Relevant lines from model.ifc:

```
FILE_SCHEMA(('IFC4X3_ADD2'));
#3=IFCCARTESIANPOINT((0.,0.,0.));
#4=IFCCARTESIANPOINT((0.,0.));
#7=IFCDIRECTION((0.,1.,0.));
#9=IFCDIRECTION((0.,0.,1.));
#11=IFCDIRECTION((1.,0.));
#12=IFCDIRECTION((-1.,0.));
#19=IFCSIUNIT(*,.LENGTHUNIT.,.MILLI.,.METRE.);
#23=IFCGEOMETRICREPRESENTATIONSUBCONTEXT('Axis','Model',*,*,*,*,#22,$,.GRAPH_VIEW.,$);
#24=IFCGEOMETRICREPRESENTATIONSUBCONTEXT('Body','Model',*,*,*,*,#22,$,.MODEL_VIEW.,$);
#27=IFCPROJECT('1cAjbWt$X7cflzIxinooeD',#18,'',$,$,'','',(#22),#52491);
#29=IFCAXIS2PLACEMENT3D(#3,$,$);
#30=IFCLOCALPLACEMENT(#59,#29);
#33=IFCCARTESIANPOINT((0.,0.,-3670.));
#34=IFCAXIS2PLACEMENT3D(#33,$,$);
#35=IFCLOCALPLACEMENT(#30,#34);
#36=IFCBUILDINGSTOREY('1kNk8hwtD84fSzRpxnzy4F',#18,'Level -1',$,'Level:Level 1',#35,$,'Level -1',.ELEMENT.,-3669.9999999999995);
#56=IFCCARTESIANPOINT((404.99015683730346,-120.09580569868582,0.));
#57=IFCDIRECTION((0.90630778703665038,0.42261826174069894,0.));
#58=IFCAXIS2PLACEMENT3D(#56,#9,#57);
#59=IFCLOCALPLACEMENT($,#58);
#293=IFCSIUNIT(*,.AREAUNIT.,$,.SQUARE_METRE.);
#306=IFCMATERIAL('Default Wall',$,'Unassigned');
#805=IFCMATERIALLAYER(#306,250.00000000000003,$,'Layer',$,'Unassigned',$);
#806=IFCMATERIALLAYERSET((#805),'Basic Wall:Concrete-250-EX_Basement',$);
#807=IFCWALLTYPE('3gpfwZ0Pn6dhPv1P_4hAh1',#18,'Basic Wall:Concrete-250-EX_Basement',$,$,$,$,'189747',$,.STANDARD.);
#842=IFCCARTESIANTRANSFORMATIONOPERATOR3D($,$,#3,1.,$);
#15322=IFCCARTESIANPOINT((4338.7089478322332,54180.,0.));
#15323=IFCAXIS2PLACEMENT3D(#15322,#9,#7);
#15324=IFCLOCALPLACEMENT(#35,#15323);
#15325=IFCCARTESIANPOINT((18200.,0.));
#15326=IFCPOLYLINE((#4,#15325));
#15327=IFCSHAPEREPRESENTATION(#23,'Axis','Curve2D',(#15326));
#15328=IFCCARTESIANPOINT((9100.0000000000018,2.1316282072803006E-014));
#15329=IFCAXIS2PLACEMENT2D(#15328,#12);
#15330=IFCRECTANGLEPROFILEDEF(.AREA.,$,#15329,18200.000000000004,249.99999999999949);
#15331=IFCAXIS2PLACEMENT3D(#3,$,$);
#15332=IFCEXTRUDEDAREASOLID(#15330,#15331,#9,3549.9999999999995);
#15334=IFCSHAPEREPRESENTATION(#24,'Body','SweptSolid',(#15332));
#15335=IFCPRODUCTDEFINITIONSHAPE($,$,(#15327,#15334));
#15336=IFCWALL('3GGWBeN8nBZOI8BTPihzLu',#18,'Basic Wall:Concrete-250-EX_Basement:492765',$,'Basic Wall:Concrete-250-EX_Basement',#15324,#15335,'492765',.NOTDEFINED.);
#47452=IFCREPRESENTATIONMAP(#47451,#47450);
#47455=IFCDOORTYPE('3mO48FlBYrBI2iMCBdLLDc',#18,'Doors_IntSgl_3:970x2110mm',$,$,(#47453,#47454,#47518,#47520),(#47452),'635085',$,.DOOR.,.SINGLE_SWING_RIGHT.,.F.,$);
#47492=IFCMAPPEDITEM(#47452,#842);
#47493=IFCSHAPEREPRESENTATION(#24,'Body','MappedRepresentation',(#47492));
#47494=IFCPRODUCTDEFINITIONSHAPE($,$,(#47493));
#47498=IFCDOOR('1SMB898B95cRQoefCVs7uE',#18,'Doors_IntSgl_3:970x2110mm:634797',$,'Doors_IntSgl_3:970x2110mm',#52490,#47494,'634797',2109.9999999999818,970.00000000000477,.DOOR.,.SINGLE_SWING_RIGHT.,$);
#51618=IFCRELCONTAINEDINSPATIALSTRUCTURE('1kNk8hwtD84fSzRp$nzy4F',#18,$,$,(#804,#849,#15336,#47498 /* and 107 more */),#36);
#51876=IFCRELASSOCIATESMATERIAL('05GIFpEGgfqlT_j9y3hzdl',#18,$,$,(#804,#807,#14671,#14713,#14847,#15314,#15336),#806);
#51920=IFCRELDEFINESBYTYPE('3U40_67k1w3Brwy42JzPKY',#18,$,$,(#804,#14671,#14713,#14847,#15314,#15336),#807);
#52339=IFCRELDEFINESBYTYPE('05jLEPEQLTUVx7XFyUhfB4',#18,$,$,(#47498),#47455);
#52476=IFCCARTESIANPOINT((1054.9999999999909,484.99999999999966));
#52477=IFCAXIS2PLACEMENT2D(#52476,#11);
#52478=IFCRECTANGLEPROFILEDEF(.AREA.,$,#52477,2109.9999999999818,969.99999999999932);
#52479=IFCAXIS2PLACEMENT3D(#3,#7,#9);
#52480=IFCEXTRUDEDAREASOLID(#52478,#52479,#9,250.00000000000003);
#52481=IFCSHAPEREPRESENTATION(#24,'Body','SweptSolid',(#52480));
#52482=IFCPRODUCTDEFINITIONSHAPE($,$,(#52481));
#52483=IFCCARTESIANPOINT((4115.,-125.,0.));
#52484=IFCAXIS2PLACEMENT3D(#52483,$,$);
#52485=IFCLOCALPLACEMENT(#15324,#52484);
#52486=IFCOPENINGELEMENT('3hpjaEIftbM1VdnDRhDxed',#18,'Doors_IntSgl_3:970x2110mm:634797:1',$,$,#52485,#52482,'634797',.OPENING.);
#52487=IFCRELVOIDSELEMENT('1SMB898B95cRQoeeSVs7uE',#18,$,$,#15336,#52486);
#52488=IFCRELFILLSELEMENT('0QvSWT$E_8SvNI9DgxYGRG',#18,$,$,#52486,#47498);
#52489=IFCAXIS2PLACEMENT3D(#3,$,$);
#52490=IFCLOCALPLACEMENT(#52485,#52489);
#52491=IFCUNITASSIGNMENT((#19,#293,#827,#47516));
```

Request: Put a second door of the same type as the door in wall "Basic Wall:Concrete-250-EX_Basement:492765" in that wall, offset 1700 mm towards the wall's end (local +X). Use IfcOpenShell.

```python
import ifcopenshell
import ifcopenshell.api.feature
import ifcopenshell.api.geometry
import ifcopenshell.api.root
import ifcopenshell.geom
import ifcopenshell.util.element
import ifcopenshell.util.placement
import ifcopenshell.util.shape

model = ifcopenshell.open("model.ifc")
settings = ifcopenshell.geom.settings()


def volume(element):
    """Net volume in cubic metres, openings subtracted."""
    shape = ifcopenshell.geom.create_shape(settings, element)
    return ifcopenshell.util.shape.get_volume(shape.geometry)


def reuse_history(source, copy):
    """copy_class also copies each property set's owner history, people and application; keep the originals."""
    for rel in copy.IsDefinedBy:
        if rel.is_a("IfcRelDefinesByProperties") and (history := rel.RelatingPropertyDefinition.OwnerHistory):
            rel.RelatingPropertyDefinition.OwnerHistory = source.OwnerHistory
            ifcopenshell.util.element.remove_deep2(model, history)


door = model.by_guid("1SMB898B95cRQoefCVs7uE")
opening = door.FillsVoids[0].RelatingOpeningElement
wall = opening.VoidsElements[0].RelatingBuildingElement
before = volume(wall)
shift = ifcopenshell.util.placement.get_local_placement(wall.ObjectPlacement)[:3, 0] * 1700.0

# copy_class copies the void relationship, type, container and properties, but no geometry.
new_opening = ifcopenshell.api.root.copy_class(model, product=opening)
new_opening.Representation = ifcopenshell.util.element.copy_deep(
    model, opening.Representation, exclude=["IfcGeometricRepresentationContext", "IfcRepresentationMap"]
)
new_opening.Name = "Doors_IntSgl_3:970x2110mm"
new_opening.Tag = None
new_door = ifcopenshell.api.root.copy_class(model, product=door)
new_door.Representation = ifcopenshell.util.element.copy_deep(
    model, door.Representation, exclude=["IfcGeometricRepresentationContext", "IfcRepresentationMap"]
)
new_door.Name = "Doors_IntSgl_3:970x2110mm"
new_door.Tag = None
reuse_history(door, new_door)
ifcopenshell.api.feature.add_filling(model, opening=new_opening, element=new_door)

for old, new in ((opening, new_opening), (door, new_door)):
    matrix = ifcopenshell.util.placement.get_local_placement(old.ObjectPlacement)
    matrix[:3, 3] += shift
    ifcopenshell.api.geometry.edit_object_placement(model, product=new, matrix=matrix, is_si=False)

after = volume(wall)

print(f"wall volume {before:.3f} -> {after:.3f} m3")

model.write("model_v2.ifc")
```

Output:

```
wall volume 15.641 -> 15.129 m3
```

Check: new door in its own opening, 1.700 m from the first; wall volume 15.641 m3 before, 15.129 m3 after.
